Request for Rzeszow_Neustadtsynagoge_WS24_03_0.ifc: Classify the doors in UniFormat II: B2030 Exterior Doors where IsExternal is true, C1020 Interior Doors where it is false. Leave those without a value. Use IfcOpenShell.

First a look at what the model holds.

```python
import ifcopenshell
import ifcopenshell.util.element

model = ifcopenshell.open("Rzeszow_Neustadtsynagoge_WS24_03_0.ifc")
print(model.schema)
print("classifications:", [c.Name for c in model.by_type("IfcClassification")])
values = [ifcopenshell.util.element.get_pset(e, "Pset_DoorCommon", "IsExternal") for e in model.by_type("IfcDoor")]
for value in (True, False, None):
    print("IsExternal", value, values.count(value))
```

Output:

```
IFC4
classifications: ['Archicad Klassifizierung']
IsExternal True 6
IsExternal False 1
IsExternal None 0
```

```python
import ifcopenshell
import ifcopenshell.api.classification
import ifcopenshell.util.element

model = ifcopenshell.open("Rzeszow_Neustadtsynagoge_WS24_03_0.ifc")

system = ifcopenshell.api.classification.add_classification(model, classification="UniFormat II")

doors = model.by_type("IfcDoor")
external = {e: ifcopenshell.util.element.get_pset(e, "Pset_DoorCommon", "IsExternal") for e in doors}
for flag, code, name in ((True, "B2030", "Exterior Doors"), (False, "C1020", "Interior Doors")):
    products = [e for e in doors if external[e] is flag]
    ifcopenshell.api.classification.add_reference(
        model, products=products, classification=system, identification=code, name=name
    )
    print(code, len(products))

model.write("Rzeszow_Neustadtsynagoge_WS24_03_0_v2.ifc")
```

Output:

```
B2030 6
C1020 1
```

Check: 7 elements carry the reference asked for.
